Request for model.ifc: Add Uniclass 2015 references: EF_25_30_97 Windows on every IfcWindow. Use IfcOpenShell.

First a look at what the model holds.

```python
import ifcopenshell

model = ifcopenshell.open("model.ifc")
print(model.schema)
print("classifications:", [c.Name for c in model.by_type("IfcClassification")])
for ifc_class in ("IfcDoor", "IfcRoof", "IfcStair", "IfcWall", "IfcWindow"):
    print(ifc_class, len(model.by_type(ifc_class)))
```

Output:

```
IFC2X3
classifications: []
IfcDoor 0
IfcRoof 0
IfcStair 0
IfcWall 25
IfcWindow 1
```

```python
import ifcopenshell
import ifcopenshell.api.classification

model = ifcopenshell.open("model.ifc")

# IFC2X3 requires Source and Edition and has no link from the project to the system.
system = model.create_entity("IfcClassification", Source="NBS", Edition="2015", Name="Uniclass 2015")

codes = {
    "IfcWindow": ("EF_25_30_97", "Windows"),
}
for ifc_class, (code, name) in codes.items():
    products = model.by_type(ifc_class)
    ifcopenshell.api.classification.add_reference(
        model, products=products, classification=system, identification=code, name=name
    )
    print(code, len(products))

model.write("model-out.ifc")
```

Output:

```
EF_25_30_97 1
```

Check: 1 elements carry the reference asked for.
